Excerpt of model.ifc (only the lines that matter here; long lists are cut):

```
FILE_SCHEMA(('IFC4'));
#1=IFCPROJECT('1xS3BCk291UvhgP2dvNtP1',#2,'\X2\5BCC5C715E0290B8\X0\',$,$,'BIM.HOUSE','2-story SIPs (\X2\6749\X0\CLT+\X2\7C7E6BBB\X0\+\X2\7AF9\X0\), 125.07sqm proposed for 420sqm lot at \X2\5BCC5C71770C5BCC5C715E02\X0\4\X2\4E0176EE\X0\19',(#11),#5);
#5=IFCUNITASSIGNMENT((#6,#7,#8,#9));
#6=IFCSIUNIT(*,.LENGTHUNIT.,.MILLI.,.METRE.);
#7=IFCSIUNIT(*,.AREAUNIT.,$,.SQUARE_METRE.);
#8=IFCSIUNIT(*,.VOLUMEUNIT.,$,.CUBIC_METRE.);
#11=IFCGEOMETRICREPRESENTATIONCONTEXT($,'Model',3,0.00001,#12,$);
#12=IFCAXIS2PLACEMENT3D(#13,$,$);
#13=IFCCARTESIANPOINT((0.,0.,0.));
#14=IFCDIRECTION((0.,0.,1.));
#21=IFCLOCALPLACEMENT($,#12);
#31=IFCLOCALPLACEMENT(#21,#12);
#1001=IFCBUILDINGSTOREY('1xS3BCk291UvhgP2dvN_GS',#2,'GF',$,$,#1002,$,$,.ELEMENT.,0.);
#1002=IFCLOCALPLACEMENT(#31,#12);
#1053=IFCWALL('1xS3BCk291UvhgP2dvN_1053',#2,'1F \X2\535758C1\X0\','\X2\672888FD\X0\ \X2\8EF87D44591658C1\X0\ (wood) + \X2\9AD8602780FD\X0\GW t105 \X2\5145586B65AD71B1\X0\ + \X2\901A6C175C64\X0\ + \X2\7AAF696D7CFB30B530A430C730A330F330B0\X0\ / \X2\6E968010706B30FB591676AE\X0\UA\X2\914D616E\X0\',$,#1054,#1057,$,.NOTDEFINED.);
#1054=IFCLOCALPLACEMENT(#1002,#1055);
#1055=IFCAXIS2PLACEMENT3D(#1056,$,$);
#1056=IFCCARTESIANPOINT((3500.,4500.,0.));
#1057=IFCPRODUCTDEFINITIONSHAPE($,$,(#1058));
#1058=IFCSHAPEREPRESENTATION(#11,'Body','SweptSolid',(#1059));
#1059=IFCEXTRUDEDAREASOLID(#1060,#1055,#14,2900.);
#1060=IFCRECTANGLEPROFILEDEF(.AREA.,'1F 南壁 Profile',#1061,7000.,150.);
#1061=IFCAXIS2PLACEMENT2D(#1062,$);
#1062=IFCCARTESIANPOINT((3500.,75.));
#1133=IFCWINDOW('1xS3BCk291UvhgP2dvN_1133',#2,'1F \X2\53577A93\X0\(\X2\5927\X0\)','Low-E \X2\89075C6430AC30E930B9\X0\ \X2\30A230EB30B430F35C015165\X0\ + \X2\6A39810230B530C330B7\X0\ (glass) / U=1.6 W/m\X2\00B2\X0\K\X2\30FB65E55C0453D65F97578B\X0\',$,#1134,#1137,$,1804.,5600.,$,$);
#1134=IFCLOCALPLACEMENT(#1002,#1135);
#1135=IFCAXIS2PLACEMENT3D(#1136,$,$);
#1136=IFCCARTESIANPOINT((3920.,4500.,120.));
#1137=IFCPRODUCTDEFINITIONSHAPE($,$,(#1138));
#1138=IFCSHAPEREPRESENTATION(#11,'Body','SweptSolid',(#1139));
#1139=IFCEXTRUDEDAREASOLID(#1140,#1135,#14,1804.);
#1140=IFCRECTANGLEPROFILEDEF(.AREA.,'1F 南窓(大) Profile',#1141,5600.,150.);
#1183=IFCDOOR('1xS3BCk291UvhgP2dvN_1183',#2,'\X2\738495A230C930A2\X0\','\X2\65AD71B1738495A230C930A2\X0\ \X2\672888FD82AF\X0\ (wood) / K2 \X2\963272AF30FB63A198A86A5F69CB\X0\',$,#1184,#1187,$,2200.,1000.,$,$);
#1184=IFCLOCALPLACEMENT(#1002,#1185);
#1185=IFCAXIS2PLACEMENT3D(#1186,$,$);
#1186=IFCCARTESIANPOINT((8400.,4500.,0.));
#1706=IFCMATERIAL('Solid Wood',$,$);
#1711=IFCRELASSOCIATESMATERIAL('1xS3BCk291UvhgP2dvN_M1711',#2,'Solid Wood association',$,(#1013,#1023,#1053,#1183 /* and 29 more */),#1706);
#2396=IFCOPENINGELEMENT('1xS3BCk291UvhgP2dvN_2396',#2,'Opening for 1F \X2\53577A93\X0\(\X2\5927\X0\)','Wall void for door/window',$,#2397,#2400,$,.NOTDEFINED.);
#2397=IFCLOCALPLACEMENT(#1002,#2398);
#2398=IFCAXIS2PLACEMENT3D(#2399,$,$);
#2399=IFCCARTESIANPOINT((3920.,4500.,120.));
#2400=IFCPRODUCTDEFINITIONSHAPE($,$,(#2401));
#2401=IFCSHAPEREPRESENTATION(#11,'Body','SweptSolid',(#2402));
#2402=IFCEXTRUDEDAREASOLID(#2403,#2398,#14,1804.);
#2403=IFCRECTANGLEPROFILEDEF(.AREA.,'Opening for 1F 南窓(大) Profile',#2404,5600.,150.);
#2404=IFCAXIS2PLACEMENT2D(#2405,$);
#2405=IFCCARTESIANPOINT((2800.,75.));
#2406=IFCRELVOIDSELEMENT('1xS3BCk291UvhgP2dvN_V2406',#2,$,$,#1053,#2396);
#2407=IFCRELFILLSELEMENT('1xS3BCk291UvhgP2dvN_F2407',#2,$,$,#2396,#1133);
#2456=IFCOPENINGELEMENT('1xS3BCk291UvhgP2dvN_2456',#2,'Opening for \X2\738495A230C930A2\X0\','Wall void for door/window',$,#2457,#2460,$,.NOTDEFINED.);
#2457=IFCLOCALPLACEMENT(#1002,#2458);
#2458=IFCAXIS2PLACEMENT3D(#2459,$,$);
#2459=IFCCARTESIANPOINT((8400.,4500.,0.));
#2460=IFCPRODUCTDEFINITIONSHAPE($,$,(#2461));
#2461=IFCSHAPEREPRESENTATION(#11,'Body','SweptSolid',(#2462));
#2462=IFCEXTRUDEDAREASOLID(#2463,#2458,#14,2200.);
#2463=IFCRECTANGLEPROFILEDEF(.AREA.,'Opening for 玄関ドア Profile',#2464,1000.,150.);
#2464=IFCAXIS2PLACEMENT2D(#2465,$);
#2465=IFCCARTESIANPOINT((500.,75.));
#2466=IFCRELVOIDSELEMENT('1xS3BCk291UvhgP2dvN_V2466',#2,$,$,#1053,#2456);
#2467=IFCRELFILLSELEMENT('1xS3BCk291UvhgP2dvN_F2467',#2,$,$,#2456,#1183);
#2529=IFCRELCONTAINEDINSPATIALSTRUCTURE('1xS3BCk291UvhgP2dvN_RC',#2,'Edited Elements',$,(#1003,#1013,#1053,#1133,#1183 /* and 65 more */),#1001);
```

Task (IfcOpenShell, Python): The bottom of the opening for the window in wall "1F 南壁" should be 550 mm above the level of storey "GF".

```python
import numpy as np
import ifcopenshell
import ifcopenshell.api.geometry
import ifcopenshell.geom
import ifcopenshell.util.element
import ifcopenshell.util.placement
import ifcopenshell.util.shape
import ifcopenshell.util.unit

model = ifcopenshell.open("model.ifc")
unit_scale = ifcopenshell.util.unit.calculate_unit_scale(model)

window = model.by_guid("1xS3BCk291UvhgP2dvN_1133")
opening = window.FillsVoids[0].RelatingOpeningElement
storey = ifcopenshell.util.element.get_container(window, ifc_class="IfcBuildingStorey")
level = ifcopenshell.util.placement.get_local_placement(storey.ObjectPlacement)[2, 3]

# The opening's origin need not be at the sill, so measure its lowest point.
shape = ifcopenshell.geom.create_shape(ifcopenshell.geom.settings(), opening)
bottom = ifcopenshell.util.shape.get_shape_bottom_elevation(shape, shape.geometry) / unit_scale
dz = level + 550.0 - bottom

shift = np.array([0.0, 0.0, dz])
# The window is not placed relative to its opening, so move both.
for product in (opening, window):
    matrix = ifcopenshell.util.placement.get_local_placement(product.ObjectPlacement)
    matrix[:3, 3] += shift
    ifcopenshell.api.geometry.edit_object_placement(model, product=product, matrix=matrix, is_si=False)

print(f"moved by {dz * unit_scale:+.3f} m")

model.write("model_edited.ifc")
```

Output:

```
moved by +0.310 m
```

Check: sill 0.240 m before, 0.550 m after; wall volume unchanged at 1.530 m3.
